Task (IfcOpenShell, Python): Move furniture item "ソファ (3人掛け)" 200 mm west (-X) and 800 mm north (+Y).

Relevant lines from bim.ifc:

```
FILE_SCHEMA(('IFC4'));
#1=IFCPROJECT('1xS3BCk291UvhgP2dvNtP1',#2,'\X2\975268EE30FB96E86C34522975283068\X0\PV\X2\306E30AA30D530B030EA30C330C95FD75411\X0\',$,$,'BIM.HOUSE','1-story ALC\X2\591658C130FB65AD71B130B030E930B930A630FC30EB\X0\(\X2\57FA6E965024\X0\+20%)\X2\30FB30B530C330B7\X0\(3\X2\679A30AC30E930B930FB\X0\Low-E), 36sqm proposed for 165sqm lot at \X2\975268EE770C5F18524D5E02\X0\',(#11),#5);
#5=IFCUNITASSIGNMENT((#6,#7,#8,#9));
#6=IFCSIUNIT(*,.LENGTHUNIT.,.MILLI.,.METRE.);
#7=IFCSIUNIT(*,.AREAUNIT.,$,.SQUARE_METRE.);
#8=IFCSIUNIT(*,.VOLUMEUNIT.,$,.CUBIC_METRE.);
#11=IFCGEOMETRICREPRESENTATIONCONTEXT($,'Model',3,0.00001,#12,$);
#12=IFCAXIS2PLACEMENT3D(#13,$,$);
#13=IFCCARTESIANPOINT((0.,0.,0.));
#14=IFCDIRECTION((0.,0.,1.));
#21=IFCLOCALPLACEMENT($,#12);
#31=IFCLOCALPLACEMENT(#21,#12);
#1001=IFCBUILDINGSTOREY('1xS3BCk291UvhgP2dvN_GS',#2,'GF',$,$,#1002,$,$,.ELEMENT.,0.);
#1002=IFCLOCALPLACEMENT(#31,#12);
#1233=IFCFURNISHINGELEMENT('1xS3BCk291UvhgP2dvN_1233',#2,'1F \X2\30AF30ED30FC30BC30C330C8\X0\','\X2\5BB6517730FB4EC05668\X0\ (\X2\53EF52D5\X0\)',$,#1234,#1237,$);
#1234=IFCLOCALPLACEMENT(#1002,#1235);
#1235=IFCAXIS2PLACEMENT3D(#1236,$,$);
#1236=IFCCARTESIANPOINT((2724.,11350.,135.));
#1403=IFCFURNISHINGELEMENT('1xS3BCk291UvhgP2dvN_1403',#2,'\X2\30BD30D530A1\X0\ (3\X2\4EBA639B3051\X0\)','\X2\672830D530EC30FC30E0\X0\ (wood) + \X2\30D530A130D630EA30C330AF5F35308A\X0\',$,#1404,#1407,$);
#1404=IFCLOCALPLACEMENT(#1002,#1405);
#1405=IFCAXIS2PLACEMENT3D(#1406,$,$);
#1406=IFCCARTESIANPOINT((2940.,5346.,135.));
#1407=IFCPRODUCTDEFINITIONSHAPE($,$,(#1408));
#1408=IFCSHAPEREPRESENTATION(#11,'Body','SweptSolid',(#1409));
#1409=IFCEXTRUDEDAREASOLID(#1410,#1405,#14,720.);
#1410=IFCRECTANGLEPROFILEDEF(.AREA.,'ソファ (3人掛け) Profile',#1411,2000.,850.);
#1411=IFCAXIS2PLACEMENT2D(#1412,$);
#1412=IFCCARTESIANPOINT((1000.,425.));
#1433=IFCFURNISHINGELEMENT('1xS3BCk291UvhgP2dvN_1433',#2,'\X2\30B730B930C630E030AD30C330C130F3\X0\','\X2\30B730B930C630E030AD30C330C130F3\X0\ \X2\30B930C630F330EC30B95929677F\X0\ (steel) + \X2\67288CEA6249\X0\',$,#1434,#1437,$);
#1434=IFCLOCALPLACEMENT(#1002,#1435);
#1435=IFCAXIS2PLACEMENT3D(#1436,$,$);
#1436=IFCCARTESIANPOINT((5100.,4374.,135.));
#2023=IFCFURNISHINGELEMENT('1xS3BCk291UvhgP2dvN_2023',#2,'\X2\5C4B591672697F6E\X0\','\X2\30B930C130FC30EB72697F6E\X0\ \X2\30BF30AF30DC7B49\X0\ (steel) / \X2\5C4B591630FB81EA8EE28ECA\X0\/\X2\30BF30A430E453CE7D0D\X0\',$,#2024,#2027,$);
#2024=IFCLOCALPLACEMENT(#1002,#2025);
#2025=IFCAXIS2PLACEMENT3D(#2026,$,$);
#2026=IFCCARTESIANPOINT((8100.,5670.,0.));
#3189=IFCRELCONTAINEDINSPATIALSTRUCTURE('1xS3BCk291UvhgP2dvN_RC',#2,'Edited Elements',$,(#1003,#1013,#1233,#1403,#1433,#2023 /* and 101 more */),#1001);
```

```python
import ifcopenshell
import ifcopenshell.api.geometry
import ifcopenshell.util.placement

model = ifcopenshell.open("bim.ifc")

item = model.by_guid("1xS3BCk291UvhgP2dvN_1403")
matrix = ifcopenshell.util.placement.get_local_placement(item.ObjectPlacement)
matrix[0, 3] -= 200.0
matrix[1, 3] += 800.0
ifcopenshell.api.geometry.edit_object_placement(model, product=item, matrix=matrix, is_si=False)

print(ifcopenshell.util.placement.get_local_placement(item.ObjectPlacement).round(3) + 0.0)

model.write("bim-out.ifc")
```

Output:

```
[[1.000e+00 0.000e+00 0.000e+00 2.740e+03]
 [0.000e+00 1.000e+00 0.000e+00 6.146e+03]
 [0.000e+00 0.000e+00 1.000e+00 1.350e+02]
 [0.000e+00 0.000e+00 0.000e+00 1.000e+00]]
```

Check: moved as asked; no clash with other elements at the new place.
